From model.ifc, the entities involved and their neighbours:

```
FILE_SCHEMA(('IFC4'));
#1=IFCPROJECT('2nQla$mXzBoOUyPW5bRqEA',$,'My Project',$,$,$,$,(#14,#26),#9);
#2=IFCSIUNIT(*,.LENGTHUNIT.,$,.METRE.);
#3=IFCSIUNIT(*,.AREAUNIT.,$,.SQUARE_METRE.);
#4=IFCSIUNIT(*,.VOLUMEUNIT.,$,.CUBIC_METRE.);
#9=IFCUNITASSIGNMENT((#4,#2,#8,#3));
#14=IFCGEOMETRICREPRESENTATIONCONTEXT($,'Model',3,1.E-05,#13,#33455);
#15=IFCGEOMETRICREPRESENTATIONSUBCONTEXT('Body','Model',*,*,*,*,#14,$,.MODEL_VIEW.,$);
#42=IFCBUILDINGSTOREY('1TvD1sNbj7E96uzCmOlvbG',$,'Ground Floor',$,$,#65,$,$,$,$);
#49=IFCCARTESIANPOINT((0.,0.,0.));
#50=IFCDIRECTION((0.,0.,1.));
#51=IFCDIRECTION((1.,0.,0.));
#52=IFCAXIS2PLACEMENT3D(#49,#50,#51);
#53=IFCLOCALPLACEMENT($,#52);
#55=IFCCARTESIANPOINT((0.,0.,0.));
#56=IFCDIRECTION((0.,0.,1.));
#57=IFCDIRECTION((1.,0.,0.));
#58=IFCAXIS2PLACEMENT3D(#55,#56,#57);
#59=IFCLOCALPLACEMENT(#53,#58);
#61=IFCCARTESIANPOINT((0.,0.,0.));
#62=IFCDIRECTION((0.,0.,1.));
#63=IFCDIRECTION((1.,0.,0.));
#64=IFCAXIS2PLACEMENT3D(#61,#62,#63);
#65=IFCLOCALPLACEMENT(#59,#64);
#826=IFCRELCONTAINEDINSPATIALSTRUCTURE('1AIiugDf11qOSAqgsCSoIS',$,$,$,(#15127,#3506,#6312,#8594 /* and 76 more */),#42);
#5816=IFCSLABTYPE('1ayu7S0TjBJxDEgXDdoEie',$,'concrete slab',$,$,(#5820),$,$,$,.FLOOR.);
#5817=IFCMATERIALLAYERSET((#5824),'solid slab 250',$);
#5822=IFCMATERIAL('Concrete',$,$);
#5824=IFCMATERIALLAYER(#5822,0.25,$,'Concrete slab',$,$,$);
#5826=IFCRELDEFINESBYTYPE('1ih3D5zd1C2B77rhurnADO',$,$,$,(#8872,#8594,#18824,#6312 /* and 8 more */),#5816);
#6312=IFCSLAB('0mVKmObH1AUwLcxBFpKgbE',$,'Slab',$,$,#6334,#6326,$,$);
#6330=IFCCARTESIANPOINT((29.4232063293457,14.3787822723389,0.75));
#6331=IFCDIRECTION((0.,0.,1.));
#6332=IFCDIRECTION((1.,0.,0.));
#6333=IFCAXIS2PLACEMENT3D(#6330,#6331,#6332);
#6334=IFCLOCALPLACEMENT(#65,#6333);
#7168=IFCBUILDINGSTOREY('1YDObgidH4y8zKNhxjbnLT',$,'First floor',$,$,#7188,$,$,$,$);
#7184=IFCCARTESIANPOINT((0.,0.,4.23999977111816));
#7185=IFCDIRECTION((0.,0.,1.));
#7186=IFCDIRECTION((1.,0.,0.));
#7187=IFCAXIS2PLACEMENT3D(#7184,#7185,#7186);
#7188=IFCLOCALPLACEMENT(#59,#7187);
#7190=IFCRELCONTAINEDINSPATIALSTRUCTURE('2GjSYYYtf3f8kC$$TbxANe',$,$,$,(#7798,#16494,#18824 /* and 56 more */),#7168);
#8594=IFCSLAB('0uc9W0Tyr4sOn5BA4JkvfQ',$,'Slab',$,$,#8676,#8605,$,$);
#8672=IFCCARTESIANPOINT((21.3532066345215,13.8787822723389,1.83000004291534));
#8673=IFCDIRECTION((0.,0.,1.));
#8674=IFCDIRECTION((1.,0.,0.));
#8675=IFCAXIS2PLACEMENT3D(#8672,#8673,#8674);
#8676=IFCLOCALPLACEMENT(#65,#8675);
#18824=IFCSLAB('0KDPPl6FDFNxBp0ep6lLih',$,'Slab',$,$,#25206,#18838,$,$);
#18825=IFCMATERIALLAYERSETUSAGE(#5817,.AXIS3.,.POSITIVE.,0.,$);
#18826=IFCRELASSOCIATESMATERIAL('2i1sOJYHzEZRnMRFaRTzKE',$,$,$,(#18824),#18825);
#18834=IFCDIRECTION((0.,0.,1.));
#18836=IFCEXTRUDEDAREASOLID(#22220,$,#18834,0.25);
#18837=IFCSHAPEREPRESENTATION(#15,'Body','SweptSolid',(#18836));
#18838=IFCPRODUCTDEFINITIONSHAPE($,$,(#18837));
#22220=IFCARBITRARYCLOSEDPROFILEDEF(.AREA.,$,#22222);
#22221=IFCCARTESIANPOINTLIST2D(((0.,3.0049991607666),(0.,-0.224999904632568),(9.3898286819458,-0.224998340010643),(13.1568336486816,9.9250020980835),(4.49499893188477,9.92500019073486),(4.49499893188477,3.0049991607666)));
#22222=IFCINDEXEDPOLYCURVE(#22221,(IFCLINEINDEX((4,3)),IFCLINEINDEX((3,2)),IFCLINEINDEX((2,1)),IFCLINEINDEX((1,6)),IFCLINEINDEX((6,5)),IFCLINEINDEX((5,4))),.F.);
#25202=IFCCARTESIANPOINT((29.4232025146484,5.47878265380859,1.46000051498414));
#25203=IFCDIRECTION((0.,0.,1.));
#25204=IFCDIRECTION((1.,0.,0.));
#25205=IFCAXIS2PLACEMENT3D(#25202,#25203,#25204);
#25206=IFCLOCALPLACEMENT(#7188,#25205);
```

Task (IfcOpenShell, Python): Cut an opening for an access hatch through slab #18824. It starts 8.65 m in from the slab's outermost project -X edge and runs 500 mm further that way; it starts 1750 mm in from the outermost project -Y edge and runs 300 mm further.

```python
import numpy as np
import ifcopenshell
import ifcopenshell.api.feature
import ifcopenshell.api.geometry
import ifcopenshell.api.root
import ifcopenshell.geom
import ifcopenshell.util.placement
import ifcopenshell.util.representation
import ifcopenshell.util.shape
import ifcopenshell.util.unit

model = ifcopenshell.open("model.ifc")
unit_scale = ifcopenshell.util.unit.calculate_unit_scale(model)
settings = ifcopenshell.geom.settings()


def volume(element):
    """Net volume in cubic metres, openings subtracted."""
    shape = ifcopenshell.geom.create_shape(settings, element)
    return ifcopenshell.util.shape.get_volume(shape.geometry)


slab = model.by_id(18824)
before = volume(slab)

# Extent in the slab's own axes, in metres. The edges named are its -X and -Y sides.
slab_shape = ifcopenshell.geom.create_shape(settings, slab)
vertices = ifcopenshell.util.shape.get_vertices(slab_shape.geometry)
x_min, y_min, bottom = vertices.min(axis=0)
top = vertices[:, 2].max()

opening = ifcopenshell.api.root.create_entity(model, ifc_class="IfcOpeningElement", name="Access hatch opening", predefined_type="OPENING")
context = ifcopenshell.util.representation.get_context(model, "Model", "Body", "MODEL_VIEW")
width, depth = 0.5, 0.3
outline = [(0.0, 0.0), (width, 0.0), (width, depth), (0.0, depth), (0.0, 0.0)]
# Overshoot both faces by 50 mm so the cut is clean.
shape = ifcopenshell.api.geometry.add_slab_representation(
    model, context=context, depth=top - bottom + 0.1, polyline=outline
)
ifcopenshell.api.geometry.assign_representation(model, product=opening, representation=shape)

matrix = ifcopenshell.util.placement.get_local_placement(slab.ObjectPlacement)
matrix[:, 3] = matrix @ np.append(np.array([x_min + 8.65, y_min + 1.75, bottom - 0.05]) / unit_scale, 1.0)
ifcopenshell.api.geometry.edit_object_placement(model, product=opening, matrix=matrix, is_si=False)
ifcopenshell.api.feature.add_feature(model, feature=opening, element=slab)

after = volume(slab)

print(f"slab volume {before:.3f} -> {after:.3f} m3")

model.write("model_edited.ifc")
```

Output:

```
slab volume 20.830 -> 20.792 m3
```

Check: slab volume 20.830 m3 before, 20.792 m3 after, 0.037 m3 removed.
